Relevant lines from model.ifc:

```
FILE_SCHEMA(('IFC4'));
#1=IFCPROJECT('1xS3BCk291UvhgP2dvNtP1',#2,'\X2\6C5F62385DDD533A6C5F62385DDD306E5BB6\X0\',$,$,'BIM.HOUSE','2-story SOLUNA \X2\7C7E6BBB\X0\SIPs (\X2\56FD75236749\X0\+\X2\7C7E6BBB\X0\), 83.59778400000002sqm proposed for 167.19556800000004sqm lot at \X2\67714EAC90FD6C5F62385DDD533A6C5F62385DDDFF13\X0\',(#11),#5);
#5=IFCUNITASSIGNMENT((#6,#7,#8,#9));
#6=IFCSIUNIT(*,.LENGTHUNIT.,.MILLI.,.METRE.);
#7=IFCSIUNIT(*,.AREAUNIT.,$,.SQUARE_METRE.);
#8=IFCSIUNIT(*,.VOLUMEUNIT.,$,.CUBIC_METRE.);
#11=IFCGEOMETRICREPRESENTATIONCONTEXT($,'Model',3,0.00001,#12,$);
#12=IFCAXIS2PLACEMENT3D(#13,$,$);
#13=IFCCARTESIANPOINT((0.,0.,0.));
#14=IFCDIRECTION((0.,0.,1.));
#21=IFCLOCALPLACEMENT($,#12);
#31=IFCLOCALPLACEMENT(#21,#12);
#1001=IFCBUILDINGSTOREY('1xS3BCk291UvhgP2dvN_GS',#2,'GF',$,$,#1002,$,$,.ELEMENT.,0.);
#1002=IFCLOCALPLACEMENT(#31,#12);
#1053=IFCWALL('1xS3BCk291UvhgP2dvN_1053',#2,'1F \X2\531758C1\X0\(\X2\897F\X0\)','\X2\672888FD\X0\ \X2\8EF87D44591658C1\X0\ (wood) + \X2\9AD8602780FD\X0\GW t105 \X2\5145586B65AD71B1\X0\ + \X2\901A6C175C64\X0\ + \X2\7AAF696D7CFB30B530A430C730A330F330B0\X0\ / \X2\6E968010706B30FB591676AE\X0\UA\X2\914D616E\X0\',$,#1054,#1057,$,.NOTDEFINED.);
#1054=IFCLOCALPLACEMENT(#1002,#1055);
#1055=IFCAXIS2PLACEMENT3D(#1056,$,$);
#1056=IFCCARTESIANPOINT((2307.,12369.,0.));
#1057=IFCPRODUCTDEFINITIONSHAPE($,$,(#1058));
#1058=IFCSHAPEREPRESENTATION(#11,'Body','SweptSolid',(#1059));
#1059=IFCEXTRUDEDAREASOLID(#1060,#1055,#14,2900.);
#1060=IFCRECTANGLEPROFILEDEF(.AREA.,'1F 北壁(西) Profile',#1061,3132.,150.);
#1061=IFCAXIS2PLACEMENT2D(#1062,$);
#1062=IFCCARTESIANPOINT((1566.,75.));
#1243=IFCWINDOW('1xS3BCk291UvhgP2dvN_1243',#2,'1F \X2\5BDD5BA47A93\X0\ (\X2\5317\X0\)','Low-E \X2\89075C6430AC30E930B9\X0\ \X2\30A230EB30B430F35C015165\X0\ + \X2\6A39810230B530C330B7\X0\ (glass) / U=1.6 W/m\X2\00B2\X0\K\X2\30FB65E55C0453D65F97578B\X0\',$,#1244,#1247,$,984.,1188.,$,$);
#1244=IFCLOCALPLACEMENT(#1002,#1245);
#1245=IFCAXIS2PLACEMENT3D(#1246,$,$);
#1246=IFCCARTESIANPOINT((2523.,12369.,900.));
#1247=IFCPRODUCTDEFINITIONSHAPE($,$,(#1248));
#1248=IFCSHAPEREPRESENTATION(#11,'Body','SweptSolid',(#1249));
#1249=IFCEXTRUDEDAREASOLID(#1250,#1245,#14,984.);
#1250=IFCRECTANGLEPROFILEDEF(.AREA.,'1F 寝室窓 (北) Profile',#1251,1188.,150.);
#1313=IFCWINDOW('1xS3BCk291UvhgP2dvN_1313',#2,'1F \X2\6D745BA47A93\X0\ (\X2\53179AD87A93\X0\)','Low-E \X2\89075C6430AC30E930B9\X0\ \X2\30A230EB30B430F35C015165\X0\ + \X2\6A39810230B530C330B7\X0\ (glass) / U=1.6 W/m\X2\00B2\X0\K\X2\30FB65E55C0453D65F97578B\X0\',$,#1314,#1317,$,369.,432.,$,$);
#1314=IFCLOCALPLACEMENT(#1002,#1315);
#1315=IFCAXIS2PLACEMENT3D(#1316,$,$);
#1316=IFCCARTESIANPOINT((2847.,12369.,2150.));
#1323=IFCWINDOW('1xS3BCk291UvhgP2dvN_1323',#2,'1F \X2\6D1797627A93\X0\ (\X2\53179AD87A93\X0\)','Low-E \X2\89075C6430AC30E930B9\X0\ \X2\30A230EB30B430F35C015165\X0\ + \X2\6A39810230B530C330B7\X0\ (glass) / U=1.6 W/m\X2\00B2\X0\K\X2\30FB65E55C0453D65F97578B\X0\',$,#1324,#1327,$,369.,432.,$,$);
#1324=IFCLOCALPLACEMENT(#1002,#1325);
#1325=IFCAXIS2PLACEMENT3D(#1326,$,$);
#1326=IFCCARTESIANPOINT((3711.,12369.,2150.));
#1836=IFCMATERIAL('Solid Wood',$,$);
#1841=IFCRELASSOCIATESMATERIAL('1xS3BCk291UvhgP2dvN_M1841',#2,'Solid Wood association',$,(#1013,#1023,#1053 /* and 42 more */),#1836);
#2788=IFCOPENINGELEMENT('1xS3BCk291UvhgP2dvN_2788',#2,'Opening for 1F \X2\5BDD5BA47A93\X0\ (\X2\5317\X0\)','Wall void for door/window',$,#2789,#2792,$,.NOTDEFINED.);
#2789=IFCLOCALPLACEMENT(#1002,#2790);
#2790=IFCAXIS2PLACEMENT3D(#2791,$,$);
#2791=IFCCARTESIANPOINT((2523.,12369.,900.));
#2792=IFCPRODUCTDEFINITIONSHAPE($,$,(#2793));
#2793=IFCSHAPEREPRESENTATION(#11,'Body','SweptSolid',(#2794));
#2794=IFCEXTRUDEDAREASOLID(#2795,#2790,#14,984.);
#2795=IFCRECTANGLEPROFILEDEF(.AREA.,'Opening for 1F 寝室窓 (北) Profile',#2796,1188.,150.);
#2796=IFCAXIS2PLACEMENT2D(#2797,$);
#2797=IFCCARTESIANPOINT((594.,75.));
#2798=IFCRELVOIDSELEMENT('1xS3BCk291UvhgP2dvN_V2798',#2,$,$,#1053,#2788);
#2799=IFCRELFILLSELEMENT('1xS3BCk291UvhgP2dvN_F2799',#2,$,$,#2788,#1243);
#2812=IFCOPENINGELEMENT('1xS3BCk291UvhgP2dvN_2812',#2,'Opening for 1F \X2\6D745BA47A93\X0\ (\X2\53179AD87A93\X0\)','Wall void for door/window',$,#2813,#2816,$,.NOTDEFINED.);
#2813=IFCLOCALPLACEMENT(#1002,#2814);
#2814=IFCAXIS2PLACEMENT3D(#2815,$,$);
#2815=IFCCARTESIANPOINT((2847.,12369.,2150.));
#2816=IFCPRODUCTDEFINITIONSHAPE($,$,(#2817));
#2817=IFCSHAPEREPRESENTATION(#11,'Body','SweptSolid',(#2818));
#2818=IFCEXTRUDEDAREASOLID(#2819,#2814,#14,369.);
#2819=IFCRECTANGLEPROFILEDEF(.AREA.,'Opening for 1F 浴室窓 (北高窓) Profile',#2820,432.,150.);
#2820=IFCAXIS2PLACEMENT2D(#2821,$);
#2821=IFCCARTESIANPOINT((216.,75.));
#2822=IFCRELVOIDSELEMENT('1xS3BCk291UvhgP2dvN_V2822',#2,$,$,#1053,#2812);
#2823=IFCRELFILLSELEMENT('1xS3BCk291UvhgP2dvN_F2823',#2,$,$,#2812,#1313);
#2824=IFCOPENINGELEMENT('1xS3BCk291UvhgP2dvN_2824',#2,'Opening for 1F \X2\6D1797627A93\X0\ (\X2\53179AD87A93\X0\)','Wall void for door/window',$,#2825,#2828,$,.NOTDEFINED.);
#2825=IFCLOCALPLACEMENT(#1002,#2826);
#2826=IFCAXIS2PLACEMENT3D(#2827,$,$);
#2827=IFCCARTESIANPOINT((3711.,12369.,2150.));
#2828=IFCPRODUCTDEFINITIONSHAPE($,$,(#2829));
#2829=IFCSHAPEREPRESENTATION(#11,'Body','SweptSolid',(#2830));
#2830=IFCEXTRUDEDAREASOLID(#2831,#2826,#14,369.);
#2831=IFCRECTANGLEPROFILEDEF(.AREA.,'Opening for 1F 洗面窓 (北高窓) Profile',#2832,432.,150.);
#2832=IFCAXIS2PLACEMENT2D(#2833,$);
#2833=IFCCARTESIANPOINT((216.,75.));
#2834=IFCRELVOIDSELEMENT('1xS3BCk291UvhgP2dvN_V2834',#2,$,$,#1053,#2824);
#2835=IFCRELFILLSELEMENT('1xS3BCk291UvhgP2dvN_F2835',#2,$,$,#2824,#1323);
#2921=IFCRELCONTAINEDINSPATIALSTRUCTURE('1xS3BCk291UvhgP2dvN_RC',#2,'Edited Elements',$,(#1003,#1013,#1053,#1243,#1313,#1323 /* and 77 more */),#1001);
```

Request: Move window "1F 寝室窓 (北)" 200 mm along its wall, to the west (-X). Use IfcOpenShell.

```python
import ifcopenshell
import ifcopenshell.api.geometry
import ifcopenshell.util.placement
import ifcopenshell.util.unit

model = ifcopenshell.open("model.ifc")
unit_scale = ifcopenshell.util.unit.calculate_unit_scale(model)

window = model.by_guid("1xS3BCk291UvhgP2dvN_1243")
opening = window.FillsVoids[0].RelatingOpeningElement
wall = opening.VoidsElements[0].RelatingBuildingElement

wall_matrix = ifcopenshell.util.placement.get_local_placement(wall.ObjectPlacement)
shift = wall_matrix[:3, 0] * -0.2 / unit_scale
before = ifcopenshell.util.placement.get_local_placement(window.ObjectPlacement)[:3, 3].copy()

# The window is not placed relative to its opening, so move both.
for product in (opening, window):
    matrix = ifcopenshell.util.placement.get_local_placement(product.ObjectPlacement)
    matrix[:3, 3] += shift
    ifcopenshell.api.geometry.edit_object_placement(model, product=product, matrix=matrix, is_si=False)

after = ifcopenshell.util.placement.get_local_placement(window.ObjectPlacement)[:3, 3]
print("window moved by", (after - before).round(3) + 0.0)

model.write("model-out.ifc")
```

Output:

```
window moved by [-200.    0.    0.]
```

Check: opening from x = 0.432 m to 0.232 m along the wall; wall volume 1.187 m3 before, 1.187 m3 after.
